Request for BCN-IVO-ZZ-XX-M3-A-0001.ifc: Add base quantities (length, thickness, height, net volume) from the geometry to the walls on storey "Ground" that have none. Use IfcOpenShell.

First a look at what the model holds.

```python
import ifcopenshell
import ifcopenshell.util.element
import ifcopenshell.util.unit

model = ifcopenshell.open("BCN-IVO-ZZ-XX-M3-A-0001.ifc")
print(model.schema)
for unit_type in ("LENGTHUNIT", "AREAUNIT", "VOLUMEUNIT"):
    print(unit_type, ifcopenshell.util.unit.calculate_unit_scale(model, unit_type))
storey = next(s for s in model.by_type("IfcBuildingStorey") if s.Name == "Ground")
walls = [e for e in ifcopenshell.util.element.get_decomposition(storey) if e.is_a("IfcWall")]
for e in sorted(walls, key=lambda e: e.id()):
    print(e.id(), e.is_a(), e.Name, list(ifcopenshell.util.element.get_psets(e, qtos_only=True)), sep=" | ")
```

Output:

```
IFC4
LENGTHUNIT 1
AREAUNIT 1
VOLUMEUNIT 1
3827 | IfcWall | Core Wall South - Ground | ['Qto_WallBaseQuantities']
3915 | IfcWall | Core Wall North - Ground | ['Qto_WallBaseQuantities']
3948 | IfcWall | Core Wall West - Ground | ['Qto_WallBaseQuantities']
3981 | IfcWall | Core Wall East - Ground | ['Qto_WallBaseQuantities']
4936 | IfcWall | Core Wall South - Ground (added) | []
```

```python
import ifcopenshell
import ifcopenshell.api.pset
import ifcopenshell.geom
import ifcopenshell.util.element
import ifcopenshell.util.shape
import ifcopenshell.util.unit

model = ifcopenshell.open("BCN-IVO-ZZ-XX-M3-A-0001.ifc")
unit_scale = ifcopenshell.util.unit.calculate_unit_scale(model)
volume_scale = ifcopenshell.util.unit.calculate_unit_scale(model, "VOLUMEUNIT")
settings = ifcopenshell.geom.settings()

storey = next(s for s in model.by_type("IfcBuildingStorey") if s.Name == "Ground")
walls = [e for e in ifcopenshell.util.element.get_decomposition(storey) if e.is_a("IfcWall")]

for e in sorted(walls, key=lambda e: e.id()):
    if ifcopenshell.util.element.get_psets(e, qtos_only=True, should_inherit=False):
        continue
    # Geometry comes back in metres, in the element's own axes.
    shape = ifcopenshell.geom.create_shape(settings, e)
    values = {
        "Length": ifcopenshell.util.shape.get_x(shape.geometry) / unit_scale,
        "Width": ifcopenshell.util.shape.get_y(shape.geometry) / unit_scale,
        "Height": ifcopenshell.util.shape.get_z(shape.geometry) / unit_scale,
        "NetVolume": ifcopenshell.util.shape.get_volume(shape.geometry) / volume_scale,
    }
    qto = ifcopenshell.api.pset.add_qto(model, product=e, name="Qto_WallBaseQuantities")
    ifcopenshell.api.pset.edit_qto(model, qto=qto, properties=values)
    print(e.id(), {k: round(v, 3) for k, v in values.items()})

model.write("BCN-IVO-ZZ-XX-M3-A-0001_rev.ifc")
```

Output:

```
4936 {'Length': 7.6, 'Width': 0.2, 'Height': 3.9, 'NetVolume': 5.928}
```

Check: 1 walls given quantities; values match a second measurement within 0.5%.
